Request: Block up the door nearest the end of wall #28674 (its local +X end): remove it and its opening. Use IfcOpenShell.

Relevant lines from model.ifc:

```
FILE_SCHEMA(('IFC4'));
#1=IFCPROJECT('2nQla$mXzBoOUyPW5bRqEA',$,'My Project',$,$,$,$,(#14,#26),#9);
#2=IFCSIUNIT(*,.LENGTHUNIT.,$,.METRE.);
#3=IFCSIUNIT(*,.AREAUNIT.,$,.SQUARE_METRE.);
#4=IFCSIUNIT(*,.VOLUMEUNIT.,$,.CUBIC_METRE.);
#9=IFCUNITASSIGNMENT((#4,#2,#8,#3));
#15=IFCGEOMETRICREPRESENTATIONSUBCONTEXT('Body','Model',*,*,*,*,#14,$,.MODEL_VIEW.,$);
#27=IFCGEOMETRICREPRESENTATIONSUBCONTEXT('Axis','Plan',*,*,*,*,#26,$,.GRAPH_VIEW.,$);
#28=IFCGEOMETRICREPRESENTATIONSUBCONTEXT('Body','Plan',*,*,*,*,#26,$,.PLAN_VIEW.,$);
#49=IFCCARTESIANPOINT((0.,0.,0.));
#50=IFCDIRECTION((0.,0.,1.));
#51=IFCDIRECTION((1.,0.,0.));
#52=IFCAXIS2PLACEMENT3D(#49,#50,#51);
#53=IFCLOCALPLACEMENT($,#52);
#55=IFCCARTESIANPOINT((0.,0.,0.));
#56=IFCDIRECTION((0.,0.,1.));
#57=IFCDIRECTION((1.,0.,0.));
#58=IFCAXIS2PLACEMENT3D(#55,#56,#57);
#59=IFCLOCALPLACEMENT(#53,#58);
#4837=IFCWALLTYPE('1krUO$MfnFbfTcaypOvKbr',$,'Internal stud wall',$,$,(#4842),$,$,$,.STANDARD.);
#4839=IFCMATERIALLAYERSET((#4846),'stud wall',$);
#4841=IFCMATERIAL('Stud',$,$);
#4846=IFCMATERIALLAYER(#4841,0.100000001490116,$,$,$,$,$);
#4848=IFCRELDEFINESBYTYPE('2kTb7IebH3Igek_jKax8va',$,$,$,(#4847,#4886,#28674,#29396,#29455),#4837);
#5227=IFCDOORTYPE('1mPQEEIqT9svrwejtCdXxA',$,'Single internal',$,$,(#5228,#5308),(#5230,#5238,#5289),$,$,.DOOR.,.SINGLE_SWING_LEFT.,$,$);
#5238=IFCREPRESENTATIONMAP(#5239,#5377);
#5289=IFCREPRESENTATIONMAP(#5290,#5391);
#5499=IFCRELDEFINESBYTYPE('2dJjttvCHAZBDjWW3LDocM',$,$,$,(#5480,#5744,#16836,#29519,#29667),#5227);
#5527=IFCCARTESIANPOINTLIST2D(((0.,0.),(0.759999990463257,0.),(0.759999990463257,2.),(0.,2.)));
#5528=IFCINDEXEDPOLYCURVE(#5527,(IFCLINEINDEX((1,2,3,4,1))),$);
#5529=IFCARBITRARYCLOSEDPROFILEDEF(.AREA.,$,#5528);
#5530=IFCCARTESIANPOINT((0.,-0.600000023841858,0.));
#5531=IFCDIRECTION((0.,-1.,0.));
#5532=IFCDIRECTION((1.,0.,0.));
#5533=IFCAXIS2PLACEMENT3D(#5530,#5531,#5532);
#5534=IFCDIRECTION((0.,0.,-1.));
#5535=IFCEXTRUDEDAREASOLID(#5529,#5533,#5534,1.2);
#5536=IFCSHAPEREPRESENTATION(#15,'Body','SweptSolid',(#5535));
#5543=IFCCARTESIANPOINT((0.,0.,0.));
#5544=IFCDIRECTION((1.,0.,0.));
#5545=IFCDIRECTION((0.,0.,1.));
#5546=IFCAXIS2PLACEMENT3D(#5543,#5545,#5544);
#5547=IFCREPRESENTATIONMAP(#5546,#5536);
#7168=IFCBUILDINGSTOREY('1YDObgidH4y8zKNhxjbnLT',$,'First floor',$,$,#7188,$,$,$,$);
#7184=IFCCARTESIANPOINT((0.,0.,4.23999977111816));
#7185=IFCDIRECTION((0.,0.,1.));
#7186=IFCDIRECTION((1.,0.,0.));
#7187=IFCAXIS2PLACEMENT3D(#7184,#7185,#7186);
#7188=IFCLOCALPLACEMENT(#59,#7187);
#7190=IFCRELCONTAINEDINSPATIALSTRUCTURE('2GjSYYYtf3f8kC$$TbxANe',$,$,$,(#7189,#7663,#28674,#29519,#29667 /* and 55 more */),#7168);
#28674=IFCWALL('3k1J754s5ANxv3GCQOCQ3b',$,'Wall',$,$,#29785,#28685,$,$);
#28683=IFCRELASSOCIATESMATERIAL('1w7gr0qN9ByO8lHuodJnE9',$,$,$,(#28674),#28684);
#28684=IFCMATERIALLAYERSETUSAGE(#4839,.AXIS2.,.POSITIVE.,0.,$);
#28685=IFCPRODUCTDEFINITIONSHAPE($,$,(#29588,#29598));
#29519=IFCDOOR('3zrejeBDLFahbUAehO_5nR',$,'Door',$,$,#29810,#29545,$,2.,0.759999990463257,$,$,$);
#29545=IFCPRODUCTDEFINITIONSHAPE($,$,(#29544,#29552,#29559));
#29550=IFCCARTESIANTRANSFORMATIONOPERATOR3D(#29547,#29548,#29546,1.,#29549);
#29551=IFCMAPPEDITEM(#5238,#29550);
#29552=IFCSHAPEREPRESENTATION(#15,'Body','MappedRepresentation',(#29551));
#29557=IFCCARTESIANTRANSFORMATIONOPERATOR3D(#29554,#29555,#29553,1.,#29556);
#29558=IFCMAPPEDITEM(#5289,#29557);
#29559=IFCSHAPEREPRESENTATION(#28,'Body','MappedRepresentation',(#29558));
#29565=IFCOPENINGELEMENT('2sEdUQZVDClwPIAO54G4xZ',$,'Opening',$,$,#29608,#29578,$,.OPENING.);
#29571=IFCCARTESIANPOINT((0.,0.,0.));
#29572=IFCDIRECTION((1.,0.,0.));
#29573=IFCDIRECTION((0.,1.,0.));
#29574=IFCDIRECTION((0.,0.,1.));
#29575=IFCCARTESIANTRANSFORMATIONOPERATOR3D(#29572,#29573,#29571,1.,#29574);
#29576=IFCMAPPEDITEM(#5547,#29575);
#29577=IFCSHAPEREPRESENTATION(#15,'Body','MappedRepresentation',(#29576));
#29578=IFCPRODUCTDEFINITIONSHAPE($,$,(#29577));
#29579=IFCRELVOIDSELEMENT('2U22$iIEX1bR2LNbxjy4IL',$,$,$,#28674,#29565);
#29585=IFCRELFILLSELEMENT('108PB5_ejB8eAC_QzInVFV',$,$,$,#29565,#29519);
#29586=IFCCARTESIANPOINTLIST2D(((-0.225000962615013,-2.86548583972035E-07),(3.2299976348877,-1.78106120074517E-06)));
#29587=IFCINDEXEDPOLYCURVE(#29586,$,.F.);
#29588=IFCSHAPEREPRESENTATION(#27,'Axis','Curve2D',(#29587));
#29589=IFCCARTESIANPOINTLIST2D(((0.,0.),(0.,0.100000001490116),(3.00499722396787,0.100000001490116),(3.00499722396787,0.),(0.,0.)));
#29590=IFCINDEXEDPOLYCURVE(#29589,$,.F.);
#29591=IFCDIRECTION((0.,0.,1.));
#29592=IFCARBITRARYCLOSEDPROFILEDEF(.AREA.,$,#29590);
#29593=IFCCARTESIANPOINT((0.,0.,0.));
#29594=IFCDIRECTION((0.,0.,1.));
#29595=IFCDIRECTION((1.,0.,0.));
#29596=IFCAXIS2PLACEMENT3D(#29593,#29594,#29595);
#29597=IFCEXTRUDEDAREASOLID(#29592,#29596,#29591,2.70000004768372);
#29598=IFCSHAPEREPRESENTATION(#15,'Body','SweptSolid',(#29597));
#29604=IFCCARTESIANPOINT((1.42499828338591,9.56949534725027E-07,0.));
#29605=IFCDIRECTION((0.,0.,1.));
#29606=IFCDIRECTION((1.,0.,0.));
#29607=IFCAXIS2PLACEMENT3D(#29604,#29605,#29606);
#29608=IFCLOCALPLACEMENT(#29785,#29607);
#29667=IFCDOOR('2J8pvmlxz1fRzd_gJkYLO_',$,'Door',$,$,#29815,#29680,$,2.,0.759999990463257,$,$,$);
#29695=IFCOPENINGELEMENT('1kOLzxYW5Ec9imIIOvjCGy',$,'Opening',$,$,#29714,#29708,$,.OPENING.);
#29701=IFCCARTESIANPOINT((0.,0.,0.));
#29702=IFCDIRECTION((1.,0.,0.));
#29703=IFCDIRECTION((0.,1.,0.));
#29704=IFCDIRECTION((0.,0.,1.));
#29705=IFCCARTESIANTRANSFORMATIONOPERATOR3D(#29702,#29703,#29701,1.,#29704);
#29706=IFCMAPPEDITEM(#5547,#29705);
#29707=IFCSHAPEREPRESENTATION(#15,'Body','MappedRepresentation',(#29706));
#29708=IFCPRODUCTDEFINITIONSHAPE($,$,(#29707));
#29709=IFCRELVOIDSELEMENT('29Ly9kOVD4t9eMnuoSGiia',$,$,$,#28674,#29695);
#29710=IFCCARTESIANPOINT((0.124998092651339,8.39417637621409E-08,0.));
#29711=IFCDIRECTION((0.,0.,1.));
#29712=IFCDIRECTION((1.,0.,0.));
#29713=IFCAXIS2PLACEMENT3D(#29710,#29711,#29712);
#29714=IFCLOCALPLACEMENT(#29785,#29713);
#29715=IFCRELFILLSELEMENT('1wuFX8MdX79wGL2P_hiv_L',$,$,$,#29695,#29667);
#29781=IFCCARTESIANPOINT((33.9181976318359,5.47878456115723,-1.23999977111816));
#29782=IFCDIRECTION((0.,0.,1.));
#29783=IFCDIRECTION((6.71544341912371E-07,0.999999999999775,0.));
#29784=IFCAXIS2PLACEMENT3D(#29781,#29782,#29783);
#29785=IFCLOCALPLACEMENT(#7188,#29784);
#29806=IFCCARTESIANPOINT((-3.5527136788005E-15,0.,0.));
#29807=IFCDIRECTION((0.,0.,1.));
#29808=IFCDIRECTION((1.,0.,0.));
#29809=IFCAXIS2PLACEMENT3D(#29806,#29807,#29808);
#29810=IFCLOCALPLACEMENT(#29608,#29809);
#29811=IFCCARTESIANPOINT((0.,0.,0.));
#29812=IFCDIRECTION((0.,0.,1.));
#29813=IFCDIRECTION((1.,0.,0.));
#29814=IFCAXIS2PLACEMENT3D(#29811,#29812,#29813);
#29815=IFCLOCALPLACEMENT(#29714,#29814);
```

```python
import ifcopenshell
import ifcopenshell.api.feature
import ifcopenshell.api.root
import ifcopenshell.geom
import ifcopenshell.util.shape

model = ifcopenshell.open("model.ifc")
settings = ifcopenshell.geom.settings()


def volume(element):
    """Net volume in cubic metres, openings subtracted."""
    shape = ifcopenshell.geom.create_shape(settings, element)
    return ifcopenshell.util.shape.get_volume(shape.geometry)


door = model.by_id(29519)
opening = door.FillsVoids[0].RelatingOpeningElement
wall = opening.VoidsElements[0].RelatingBuildingElement
before = volume(wall)

ifcopenshell.api.root.remove_product(model, product=door)
ifcopenshell.api.feature.remove_feature(model, feature=opening)

after = volume(wall)

print(f"wall volume {before:.3f} -> {after:.3f} m3")

model.write("model_v2.ifc")
```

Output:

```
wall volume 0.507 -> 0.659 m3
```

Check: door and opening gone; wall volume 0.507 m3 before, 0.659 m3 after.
